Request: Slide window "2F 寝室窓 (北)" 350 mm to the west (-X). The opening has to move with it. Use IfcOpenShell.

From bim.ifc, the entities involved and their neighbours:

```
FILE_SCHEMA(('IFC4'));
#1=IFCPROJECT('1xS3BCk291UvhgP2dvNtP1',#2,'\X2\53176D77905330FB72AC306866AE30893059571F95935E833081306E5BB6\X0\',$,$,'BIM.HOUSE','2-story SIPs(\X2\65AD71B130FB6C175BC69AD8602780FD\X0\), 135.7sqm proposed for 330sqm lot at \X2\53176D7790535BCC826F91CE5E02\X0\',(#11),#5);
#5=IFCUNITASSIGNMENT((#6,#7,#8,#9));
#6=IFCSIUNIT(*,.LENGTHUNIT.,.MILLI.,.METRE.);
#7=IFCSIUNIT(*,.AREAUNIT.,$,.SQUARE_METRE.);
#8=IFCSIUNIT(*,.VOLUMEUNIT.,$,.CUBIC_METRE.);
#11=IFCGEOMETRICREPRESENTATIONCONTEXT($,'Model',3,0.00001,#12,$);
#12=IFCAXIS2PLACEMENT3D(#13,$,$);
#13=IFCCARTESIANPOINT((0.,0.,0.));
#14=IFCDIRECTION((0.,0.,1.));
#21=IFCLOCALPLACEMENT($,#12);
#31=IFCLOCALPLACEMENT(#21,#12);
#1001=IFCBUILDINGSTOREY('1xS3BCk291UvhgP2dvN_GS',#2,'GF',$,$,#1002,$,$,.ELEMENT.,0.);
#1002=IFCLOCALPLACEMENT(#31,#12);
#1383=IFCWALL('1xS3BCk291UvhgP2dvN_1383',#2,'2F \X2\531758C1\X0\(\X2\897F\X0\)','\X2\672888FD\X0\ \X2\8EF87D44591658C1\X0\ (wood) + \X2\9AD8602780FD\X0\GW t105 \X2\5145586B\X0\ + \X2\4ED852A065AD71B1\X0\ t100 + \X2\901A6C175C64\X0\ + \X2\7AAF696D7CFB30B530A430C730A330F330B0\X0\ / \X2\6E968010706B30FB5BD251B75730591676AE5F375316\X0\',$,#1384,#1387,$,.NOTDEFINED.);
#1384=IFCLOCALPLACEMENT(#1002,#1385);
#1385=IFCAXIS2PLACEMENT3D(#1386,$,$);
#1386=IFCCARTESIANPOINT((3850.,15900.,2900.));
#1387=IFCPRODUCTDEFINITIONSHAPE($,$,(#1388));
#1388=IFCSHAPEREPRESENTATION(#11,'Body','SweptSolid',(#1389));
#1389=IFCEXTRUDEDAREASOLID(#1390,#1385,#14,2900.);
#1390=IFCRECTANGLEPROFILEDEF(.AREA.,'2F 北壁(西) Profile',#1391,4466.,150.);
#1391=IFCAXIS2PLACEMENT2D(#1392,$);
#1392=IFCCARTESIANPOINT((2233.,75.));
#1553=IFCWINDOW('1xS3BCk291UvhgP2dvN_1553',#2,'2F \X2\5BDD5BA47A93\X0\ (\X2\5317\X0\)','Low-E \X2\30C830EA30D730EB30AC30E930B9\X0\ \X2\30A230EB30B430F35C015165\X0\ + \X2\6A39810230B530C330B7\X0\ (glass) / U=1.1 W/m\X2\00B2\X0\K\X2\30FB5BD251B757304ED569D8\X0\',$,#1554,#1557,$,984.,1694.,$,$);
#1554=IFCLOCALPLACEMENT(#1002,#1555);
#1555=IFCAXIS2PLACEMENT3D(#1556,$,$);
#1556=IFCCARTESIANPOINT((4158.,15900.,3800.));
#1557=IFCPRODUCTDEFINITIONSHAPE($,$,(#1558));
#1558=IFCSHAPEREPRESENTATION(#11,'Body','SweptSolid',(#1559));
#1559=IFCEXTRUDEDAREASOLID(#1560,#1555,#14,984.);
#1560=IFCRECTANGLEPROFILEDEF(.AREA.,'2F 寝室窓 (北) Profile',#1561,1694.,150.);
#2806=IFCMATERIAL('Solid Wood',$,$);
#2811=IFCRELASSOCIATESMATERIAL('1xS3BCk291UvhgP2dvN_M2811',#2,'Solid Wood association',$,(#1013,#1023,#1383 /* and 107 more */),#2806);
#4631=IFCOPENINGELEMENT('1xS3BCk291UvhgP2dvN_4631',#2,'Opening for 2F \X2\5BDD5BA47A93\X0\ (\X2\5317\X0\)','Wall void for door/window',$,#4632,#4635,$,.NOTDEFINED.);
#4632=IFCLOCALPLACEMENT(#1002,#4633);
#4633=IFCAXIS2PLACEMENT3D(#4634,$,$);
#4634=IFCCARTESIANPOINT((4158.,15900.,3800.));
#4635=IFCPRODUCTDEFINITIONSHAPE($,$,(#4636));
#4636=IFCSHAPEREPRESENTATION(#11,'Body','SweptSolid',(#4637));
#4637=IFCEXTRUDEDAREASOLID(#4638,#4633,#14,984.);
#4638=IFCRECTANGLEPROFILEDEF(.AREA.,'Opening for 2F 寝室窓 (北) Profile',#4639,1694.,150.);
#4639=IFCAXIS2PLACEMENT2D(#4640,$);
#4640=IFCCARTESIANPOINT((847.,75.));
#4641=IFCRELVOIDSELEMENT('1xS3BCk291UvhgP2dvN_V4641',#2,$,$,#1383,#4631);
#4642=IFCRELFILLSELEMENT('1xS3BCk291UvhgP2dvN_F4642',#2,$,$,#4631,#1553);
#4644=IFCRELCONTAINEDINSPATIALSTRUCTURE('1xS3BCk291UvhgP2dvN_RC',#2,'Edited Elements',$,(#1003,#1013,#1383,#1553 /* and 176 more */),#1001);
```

```python
import ifcopenshell
import ifcopenshell.api.geometry
import ifcopenshell.util.placement
import ifcopenshell.util.unit

model = ifcopenshell.open("bim.ifc")
unit_scale = ifcopenshell.util.unit.calculate_unit_scale(model)

window = model.by_guid("1xS3BCk291UvhgP2dvN_1553")
opening = window.FillsVoids[0].RelatingOpeningElement
wall = opening.VoidsElements[0].RelatingBuildingElement

wall_matrix = ifcopenshell.util.placement.get_local_placement(wall.ObjectPlacement)
shift = wall_matrix[:3, 0] * -0.35 / unit_scale
before = ifcopenshell.util.placement.get_local_placement(window.ObjectPlacement)[:3, 3].copy()

# The window is not placed relative to its opening, so move both.
for product in (opening, window):
    matrix = ifcopenshell.util.placement.get_local_placement(product.ObjectPlacement)
    matrix[:3, 3] += shift
    ifcopenshell.api.geometry.edit_object_placement(model, product=product, matrix=matrix, is_si=False)

after = ifcopenshell.util.placement.get_local_placement(window.ObjectPlacement)[:3, 3]
print("window moved by", (after - before).round(3) + 0.0)

model.write("bim_edited.ifc")
```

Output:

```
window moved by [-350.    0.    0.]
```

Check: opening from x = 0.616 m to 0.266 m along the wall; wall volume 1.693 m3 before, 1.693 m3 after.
